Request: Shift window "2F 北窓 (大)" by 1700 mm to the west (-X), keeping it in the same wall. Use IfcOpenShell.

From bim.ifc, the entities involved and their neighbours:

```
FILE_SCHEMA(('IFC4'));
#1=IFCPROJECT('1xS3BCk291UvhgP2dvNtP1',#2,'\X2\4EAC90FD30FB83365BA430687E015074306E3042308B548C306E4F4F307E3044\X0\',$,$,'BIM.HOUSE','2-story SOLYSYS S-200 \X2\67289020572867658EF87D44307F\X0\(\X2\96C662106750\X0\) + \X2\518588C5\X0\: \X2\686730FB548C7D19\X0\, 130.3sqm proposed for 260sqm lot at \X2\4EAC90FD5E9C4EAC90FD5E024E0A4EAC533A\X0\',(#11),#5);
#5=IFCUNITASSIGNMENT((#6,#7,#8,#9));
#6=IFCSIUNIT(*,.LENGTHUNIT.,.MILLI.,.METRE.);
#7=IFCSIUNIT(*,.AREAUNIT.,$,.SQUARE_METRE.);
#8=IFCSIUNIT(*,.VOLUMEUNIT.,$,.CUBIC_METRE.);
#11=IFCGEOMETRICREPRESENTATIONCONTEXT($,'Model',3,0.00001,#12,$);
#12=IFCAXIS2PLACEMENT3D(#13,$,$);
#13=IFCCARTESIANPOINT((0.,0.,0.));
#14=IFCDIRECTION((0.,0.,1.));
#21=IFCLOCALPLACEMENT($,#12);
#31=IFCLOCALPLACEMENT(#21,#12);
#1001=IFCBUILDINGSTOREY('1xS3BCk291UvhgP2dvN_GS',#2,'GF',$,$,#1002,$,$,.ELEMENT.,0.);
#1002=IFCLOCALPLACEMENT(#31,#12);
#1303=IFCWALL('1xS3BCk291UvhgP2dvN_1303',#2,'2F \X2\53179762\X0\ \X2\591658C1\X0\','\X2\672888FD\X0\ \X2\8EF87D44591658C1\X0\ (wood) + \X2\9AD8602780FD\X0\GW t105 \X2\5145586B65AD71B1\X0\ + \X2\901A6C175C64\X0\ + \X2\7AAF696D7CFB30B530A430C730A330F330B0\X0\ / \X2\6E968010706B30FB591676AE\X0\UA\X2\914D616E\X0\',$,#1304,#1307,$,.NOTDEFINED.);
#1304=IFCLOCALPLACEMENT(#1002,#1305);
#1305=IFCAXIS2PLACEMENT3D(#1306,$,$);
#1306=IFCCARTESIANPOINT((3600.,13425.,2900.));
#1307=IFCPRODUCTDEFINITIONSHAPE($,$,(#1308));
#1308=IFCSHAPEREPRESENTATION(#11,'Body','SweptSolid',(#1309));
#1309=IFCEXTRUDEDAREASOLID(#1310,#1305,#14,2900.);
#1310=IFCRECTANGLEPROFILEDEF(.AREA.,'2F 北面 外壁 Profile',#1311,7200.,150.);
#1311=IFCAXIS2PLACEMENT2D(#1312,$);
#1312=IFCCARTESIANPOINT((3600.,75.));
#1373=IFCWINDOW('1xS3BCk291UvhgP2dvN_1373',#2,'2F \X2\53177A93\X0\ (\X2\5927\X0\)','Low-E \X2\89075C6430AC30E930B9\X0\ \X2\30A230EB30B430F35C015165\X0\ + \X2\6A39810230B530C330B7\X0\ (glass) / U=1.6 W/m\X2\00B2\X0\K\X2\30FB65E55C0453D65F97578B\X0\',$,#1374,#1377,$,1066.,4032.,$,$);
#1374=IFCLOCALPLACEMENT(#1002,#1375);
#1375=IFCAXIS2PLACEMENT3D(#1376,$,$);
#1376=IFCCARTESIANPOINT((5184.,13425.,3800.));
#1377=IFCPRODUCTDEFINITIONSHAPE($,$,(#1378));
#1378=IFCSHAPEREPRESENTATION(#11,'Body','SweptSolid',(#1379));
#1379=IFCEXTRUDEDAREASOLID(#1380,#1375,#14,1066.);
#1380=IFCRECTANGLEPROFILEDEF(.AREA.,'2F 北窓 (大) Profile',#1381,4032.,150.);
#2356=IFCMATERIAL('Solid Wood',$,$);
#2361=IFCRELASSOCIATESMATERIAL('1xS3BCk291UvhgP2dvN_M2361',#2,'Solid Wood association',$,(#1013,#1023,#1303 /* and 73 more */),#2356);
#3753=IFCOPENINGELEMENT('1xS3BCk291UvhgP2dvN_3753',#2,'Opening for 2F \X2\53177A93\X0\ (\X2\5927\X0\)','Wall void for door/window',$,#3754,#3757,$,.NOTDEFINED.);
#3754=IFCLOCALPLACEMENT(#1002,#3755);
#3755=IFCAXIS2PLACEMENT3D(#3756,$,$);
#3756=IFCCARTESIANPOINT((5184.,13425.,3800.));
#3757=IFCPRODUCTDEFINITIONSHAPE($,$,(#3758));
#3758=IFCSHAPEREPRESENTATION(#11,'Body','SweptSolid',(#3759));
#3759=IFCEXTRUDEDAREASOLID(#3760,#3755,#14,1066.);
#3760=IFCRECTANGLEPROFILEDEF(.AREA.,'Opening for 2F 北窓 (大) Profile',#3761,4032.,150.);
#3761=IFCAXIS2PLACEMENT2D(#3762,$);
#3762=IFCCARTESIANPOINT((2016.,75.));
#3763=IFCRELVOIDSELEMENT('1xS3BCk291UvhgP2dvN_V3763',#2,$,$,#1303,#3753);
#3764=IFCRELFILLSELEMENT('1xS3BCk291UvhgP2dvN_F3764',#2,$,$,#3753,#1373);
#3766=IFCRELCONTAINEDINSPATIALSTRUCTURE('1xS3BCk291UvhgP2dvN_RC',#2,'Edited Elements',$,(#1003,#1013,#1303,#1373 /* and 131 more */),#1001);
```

```python
import ifcopenshell
import ifcopenshell.api.geometry
import ifcopenshell.util.placement

model = ifcopenshell.open("bim.ifc")

window = model.by_guid("1xS3BCk291UvhgP2dvN_1373")
opening = window.FillsVoids[0].RelatingOpeningElement
wall = opening.VoidsElements[0].RelatingBuildingElement

wall_matrix = ifcopenshell.util.placement.get_local_placement(wall.ObjectPlacement)
shift = wall_matrix[:3, 0] * -1700.0
before = ifcopenshell.util.placement.get_local_placement(window.ObjectPlacement)[:3, 3].copy()

# The window is not placed relative to its opening, so move both.
for product in (opening, window):
    matrix = ifcopenshell.util.placement.get_local_placement(product.ObjectPlacement)
    matrix[:3, 3] += shift
    ifcopenshell.api.geometry.edit_object_placement(model, product=product, matrix=matrix, is_si=False)

after = ifcopenshell.util.placement.get_local_placement(window.ObjectPlacement)[:3, 3]
print("window moved by", (after - before).round(3) + 0.0)

model.write("bim_updated.ifc")
```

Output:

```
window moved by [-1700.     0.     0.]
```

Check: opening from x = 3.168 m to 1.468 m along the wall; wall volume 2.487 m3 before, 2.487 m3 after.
